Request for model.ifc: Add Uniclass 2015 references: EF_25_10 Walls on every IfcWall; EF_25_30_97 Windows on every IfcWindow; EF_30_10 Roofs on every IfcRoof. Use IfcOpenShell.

First a look at what the model holds.

```python
import ifcopenshell

model = ifcopenshell.open("model.ifc")
print(model.schema)
print("classifications:", [c.Name for c in model.by_type("IfcClassification")])
for ifc_class in ("IfcDoor", "IfcRoof", "IfcStair", "IfcWall", "IfcWindow"):
    print(ifc_class, len(model.by_type(ifc_class)))
```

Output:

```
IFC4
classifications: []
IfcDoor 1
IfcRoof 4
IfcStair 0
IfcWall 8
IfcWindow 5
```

```python
import ifcopenshell
import ifcopenshell.api.classification

model = ifcopenshell.open("model.ifc")

system = ifcopenshell.api.classification.add_classification(model, classification="Uniclass 2015")

codes = {
    "IfcWall": ("EF_25_10", "Walls"),
    "IfcWindow": ("EF_25_30_97", "Windows"),
    "IfcRoof": ("EF_30_10", "Roofs"),
}
for ifc_class, (code, name) in codes.items():
    products = model.by_type(ifc_class)
    ifcopenshell.api.classification.add_reference(
        model, products=products, classification=system, identification=code, name=name
    )
    print(code, len(products))

model.write("model_updated.ifc")
```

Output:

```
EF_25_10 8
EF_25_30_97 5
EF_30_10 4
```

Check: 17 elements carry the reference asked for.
